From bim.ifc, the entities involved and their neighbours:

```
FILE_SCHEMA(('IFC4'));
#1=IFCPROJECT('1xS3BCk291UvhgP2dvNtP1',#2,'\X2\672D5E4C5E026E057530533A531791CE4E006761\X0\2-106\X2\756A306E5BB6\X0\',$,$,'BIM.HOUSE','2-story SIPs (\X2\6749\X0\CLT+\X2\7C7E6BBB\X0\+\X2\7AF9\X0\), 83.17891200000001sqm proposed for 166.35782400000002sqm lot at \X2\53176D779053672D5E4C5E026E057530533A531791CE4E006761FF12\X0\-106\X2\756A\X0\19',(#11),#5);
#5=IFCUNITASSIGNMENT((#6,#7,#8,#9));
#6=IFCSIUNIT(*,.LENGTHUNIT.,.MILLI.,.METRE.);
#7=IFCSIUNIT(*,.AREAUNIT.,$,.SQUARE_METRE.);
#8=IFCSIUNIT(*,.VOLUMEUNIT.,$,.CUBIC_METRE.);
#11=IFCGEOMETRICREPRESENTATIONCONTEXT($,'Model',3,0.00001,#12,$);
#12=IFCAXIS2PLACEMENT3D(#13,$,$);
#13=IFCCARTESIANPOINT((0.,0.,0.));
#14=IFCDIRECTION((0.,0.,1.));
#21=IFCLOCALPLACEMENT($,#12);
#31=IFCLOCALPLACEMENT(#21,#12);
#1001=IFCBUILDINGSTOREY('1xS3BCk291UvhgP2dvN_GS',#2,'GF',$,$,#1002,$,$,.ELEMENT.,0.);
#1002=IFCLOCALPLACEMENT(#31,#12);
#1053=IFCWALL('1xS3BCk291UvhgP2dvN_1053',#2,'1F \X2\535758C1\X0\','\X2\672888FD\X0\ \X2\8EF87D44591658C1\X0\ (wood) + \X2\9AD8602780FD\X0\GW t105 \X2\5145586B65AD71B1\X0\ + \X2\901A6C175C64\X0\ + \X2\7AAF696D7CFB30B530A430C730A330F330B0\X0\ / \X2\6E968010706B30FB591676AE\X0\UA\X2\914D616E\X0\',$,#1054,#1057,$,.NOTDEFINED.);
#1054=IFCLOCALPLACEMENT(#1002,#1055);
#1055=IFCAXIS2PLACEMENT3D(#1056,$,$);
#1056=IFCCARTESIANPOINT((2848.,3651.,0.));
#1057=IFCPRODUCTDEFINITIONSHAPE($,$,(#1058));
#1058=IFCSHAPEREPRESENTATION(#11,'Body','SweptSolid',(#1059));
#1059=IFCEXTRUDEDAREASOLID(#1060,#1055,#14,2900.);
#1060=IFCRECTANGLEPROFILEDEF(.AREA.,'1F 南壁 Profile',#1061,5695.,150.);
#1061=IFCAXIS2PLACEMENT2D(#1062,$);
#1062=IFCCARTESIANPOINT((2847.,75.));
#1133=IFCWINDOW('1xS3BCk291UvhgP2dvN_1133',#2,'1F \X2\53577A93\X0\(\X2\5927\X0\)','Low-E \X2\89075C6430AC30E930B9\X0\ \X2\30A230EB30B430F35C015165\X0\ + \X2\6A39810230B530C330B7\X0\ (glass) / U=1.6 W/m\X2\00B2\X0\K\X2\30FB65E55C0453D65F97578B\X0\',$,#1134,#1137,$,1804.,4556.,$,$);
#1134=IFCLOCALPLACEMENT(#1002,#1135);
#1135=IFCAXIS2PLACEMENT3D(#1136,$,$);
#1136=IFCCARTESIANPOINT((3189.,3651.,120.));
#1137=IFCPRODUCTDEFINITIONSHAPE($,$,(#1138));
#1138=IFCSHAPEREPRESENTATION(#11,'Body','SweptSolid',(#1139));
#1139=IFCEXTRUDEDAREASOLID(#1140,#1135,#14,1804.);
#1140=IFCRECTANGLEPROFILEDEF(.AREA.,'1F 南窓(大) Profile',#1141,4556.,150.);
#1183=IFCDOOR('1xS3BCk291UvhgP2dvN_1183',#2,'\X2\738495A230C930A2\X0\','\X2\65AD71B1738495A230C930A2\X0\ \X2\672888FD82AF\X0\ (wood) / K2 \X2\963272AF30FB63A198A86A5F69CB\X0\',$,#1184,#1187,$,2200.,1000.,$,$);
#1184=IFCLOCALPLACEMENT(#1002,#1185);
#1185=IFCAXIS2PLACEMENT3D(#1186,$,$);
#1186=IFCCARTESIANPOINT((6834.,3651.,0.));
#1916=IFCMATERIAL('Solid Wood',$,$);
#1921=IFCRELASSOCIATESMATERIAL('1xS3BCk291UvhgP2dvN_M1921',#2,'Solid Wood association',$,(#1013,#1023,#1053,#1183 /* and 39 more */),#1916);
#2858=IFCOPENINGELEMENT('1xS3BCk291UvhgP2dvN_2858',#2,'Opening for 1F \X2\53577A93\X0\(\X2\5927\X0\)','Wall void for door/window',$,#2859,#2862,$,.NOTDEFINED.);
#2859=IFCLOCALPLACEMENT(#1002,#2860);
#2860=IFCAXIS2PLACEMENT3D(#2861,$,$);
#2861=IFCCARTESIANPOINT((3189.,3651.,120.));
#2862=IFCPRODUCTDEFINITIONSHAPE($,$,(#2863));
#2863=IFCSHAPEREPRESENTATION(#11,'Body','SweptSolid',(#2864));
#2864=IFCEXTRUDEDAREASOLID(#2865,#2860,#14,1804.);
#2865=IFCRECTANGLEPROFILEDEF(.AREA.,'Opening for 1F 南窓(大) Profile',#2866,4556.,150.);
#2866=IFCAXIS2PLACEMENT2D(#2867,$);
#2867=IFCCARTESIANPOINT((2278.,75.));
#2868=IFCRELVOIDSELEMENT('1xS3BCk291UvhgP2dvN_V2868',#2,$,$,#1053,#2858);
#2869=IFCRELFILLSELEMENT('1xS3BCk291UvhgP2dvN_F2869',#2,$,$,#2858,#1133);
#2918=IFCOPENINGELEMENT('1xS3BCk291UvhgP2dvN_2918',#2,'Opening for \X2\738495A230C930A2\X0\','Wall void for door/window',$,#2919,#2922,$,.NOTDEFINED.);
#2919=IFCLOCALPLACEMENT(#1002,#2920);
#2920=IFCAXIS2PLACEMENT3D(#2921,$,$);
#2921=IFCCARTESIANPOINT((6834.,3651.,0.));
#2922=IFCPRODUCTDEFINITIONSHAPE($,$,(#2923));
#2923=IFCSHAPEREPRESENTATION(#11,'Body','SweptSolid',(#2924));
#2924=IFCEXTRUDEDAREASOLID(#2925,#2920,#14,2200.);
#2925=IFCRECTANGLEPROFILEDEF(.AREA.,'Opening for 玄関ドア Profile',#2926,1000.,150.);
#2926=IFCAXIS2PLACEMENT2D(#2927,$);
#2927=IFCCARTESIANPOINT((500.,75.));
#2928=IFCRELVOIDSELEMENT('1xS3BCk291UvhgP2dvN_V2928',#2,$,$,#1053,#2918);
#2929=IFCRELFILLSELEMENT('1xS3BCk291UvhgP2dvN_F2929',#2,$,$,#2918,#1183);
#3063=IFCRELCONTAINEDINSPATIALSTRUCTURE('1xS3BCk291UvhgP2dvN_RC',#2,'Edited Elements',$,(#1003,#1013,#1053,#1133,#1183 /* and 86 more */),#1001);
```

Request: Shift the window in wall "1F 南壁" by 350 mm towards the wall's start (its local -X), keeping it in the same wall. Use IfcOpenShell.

```python
import ifcopenshell
import ifcopenshell.api.geometry
import ifcopenshell.util.placement

model = ifcopenshell.open("bim.ifc")

window = model.by_id(1133)
opening = window.FillsVoids[0].RelatingOpeningElement
wall = opening.VoidsElements[0].RelatingBuildingElement

wall_matrix = ifcopenshell.util.placement.get_local_placement(wall.ObjectPlacement)
shift = wall_matrix[:3, 0] * -350.0
before = ifcopenshell.util.placement.get_local_placement(window.ObjectPlacement)[:3, 3].copy()

# The window is not placed relative to its opening, so move both.
for product in (opening, window):
    matrix = ifcopenshell.util.placement.get_local_placement(product.ObjectPlacement)
    matrix[:3, 3] += shift
    ifcopenshell.api.geometry.edit_object_placement(model, product=product, matrix=matrix, is_si=False)

after = ifcopenshell.util.placement.get_local_placement(window.ObjectPlacement)[:3, 3]
print("window moved by", (after - before).round(3) + 0.0)

model.write("bim_edited.ifc")
```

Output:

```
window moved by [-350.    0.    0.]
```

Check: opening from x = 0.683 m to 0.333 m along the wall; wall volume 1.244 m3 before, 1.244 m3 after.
